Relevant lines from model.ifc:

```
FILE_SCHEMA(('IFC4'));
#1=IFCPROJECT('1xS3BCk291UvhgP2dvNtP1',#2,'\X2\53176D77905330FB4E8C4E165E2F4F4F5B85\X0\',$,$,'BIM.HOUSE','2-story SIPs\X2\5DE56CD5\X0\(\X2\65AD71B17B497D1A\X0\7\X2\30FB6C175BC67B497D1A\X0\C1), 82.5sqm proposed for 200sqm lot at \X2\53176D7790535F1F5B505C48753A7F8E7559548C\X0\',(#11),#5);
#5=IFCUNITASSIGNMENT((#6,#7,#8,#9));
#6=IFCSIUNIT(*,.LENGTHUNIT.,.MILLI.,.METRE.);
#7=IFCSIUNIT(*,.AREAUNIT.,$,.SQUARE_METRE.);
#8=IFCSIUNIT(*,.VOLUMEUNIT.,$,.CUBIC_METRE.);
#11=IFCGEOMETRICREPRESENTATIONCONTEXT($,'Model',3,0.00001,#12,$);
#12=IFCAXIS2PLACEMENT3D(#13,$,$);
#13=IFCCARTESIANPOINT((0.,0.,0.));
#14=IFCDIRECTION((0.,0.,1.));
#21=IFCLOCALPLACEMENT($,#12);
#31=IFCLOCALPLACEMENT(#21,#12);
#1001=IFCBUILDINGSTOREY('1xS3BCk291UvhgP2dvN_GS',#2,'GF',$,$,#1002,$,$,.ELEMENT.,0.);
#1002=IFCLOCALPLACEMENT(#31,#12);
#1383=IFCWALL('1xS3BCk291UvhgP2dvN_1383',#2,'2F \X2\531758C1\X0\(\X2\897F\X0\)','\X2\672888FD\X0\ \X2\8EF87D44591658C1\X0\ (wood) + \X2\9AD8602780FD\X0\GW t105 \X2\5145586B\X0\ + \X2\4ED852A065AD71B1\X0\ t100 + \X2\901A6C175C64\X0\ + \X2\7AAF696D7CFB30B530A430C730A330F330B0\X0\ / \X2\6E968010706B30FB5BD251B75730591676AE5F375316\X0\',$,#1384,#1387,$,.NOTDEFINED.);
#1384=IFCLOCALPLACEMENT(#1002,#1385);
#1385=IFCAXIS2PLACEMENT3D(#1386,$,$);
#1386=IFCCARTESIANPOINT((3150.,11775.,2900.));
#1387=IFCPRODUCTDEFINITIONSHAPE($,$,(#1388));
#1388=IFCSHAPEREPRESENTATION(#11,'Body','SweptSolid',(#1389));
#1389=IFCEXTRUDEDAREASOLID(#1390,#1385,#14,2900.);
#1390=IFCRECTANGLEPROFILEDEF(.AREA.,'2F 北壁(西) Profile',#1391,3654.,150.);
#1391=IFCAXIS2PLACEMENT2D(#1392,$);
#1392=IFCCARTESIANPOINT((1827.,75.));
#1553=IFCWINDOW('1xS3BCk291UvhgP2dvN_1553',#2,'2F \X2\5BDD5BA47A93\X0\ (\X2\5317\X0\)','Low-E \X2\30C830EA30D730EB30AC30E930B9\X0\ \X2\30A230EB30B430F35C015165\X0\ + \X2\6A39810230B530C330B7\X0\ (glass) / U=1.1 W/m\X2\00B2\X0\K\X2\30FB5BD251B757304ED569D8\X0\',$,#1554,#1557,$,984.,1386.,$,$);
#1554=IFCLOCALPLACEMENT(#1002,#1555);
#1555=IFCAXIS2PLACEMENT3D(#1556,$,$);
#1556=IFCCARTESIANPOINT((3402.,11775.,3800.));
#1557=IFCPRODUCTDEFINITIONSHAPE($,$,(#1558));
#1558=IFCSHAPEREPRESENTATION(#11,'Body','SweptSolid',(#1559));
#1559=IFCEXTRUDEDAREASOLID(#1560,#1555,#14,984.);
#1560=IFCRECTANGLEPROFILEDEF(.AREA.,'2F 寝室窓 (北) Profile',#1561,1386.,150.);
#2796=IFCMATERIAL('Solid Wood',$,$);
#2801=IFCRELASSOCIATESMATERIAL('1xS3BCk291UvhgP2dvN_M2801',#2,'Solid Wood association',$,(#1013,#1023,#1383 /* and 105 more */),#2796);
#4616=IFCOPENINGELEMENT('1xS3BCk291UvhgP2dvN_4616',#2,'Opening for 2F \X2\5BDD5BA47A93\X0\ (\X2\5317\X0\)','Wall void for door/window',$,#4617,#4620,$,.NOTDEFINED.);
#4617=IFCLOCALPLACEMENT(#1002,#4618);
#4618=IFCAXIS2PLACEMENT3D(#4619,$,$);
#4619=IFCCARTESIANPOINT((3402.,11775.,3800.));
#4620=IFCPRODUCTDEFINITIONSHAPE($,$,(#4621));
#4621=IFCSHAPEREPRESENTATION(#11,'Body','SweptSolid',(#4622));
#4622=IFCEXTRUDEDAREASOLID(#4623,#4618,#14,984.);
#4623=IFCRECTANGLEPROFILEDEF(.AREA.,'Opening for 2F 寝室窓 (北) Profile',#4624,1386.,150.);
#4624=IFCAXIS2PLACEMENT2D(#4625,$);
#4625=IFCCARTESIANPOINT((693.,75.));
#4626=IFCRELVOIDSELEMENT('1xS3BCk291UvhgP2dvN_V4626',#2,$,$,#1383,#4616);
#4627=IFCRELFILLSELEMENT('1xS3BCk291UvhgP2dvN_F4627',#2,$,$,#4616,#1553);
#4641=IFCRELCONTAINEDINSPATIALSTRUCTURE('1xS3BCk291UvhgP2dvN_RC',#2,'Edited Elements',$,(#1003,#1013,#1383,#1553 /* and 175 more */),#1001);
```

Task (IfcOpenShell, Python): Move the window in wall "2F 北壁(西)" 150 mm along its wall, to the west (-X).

```python
import ifcopenshell
import ifcopenshell.api.geometry
import ifcopenshell.util.placement
import ifcopenshell.util.unit

model = ifcopenshell.open("model.ifc")
unit_scale = ifcopenshell.util.unit.calculate_unit_scale(model)

window = model.by_guid("1xS3BCk291UvhgP2dvN_1553")
opening = window.FillsVoids[0].RelatingOpeningElement
wall = opening.VoidsElements[0].RelatingBuildingElement

wall_matrix = ifcopenshell.util.placement.get_local_placement(wall.ObjectPlacement)
shift = wall_matrix[:3, 0] * -0.15 / unit_scale
before = ifcopenshell.util.placement.get_local_placement(window.ObjectPlacement)[:3, 3].copy()

# The window is not placed relative to its opening, so move both.
for product in (opening, window):
    matrix = ifcopenshell.util.placement.get_local_placement(product.ObjectPlacement)
    matrix[:3, 3] += shift
    ifcopenshell.api.geometry.edit_object_placement(model, product=product, matrix=matrix, is_si=False)

after = ifcopenshell.util.placement.get_local_placement(window.ObjectPlacement)[:3, 3]
print("window moved by", (after - before).round(3) + 0.0)

model.write("model_edited.ifc")
```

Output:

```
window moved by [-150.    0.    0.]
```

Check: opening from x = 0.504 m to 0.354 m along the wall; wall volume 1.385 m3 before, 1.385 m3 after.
